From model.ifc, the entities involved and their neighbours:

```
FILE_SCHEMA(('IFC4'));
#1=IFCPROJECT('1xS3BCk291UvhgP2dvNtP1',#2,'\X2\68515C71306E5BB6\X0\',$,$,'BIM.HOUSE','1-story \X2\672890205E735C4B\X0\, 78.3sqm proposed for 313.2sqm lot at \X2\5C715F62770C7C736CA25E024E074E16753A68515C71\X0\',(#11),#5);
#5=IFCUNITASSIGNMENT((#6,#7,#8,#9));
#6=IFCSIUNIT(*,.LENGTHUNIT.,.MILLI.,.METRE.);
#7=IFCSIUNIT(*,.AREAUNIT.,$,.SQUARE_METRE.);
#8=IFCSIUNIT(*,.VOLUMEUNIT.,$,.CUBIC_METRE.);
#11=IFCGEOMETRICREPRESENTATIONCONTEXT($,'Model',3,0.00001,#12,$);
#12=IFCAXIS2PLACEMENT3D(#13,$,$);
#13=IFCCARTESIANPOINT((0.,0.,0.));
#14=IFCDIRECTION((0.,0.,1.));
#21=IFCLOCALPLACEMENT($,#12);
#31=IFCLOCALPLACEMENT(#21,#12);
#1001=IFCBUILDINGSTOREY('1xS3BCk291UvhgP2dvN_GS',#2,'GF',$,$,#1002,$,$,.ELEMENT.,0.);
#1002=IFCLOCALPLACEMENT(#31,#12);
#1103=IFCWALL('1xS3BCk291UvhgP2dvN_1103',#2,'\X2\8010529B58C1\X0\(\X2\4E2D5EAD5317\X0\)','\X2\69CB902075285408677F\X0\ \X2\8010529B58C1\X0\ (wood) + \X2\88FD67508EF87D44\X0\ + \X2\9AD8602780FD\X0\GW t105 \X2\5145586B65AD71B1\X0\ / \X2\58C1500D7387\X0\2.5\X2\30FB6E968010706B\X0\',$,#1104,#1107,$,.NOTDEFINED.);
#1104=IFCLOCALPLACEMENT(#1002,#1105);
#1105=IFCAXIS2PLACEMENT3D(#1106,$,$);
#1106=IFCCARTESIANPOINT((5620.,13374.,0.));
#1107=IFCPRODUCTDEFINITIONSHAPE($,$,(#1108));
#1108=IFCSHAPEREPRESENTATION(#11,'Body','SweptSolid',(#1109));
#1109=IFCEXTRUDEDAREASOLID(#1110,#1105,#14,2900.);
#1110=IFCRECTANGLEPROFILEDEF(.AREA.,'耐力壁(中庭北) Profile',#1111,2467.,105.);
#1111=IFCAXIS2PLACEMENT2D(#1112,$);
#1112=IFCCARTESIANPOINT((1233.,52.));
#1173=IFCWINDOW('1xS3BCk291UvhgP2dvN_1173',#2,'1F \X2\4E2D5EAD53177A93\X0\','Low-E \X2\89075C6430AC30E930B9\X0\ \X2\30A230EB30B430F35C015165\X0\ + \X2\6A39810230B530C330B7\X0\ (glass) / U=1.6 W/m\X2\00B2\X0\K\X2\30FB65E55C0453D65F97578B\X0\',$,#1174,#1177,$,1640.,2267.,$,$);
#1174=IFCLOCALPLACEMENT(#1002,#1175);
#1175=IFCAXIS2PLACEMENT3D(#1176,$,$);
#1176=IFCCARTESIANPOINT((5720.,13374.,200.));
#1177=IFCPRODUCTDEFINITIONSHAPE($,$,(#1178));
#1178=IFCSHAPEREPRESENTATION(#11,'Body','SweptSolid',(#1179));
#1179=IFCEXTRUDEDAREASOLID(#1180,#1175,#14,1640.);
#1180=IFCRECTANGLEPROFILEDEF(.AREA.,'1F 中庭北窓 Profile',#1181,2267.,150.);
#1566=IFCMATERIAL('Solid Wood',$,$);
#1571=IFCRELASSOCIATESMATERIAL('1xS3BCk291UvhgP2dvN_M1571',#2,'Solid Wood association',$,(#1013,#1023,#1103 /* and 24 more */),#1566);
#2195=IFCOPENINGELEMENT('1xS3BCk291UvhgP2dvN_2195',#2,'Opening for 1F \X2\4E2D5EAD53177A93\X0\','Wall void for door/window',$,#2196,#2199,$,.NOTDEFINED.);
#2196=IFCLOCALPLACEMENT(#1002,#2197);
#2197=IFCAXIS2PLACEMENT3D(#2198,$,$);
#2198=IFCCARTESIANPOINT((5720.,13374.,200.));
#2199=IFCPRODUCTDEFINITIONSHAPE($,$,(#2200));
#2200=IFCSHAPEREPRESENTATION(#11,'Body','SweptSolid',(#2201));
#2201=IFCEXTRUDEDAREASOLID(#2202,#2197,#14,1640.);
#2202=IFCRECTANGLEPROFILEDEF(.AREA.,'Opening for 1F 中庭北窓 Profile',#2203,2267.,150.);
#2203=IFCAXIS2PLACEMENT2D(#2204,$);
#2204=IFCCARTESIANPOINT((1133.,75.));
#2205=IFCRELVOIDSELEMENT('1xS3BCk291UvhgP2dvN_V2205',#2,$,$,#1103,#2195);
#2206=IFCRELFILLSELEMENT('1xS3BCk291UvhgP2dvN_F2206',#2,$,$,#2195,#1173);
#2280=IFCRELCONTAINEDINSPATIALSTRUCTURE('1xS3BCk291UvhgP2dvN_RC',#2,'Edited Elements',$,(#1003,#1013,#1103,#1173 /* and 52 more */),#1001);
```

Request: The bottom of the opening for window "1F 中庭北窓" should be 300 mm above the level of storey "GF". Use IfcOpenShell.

```python
import numpy as np
import ifcopenshell
import ifcopenshell.api.geometry
import ifcopenshell.geom
import ifcopenshell.util.element
import ifcopenshell.util.placement
import ifcopenshell.util.shape
import ifcopenshell.util.unit

model = ifcopenshell.open("model.ifc")
unit_scale = ifcopenshell.util.unit.calculate_unit_scale(model)

window = model.by_id(1173)
opening = window.FillsVoids[0].RelatingOpeningElement
storey = ifcopenshell.util.element.get_container(window, ifc_class="IfcBuildingStorey")
level = ifcopenshell.util.placement.get_local_placement(storey.ObjectPlacement)[2, 3]

# The opening's origin need not be at the sill, so measure its lowest point.
shape = ifcopenshell.geom.create_shape(ifcopenshell.geom.settings(), opening)
bottom = ifcopenshell.util.shape.get_shape_bottom_elevation(shape, shape.geometry) / unit_scale
dz = level + 300.0 - bottom

shift = np.array([0.0, 0.0, dz])
# The window is not placed relative to its opening, so move both.
for product in (opening, window):
    matrix = ifcopenshell.util.placement.get_local_placement(product.ObjectPlacement)
    matrix[:3, 3] += shift
    ifcopenshell.api.geometry.edit_object_placement(model, product=product, matrix=matrix, is_si=False)

print(f"moved by {dz * unit_scale:+.3f} m")

model.write("model-out.ifc")
```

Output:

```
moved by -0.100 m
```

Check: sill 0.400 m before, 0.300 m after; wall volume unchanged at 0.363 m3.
